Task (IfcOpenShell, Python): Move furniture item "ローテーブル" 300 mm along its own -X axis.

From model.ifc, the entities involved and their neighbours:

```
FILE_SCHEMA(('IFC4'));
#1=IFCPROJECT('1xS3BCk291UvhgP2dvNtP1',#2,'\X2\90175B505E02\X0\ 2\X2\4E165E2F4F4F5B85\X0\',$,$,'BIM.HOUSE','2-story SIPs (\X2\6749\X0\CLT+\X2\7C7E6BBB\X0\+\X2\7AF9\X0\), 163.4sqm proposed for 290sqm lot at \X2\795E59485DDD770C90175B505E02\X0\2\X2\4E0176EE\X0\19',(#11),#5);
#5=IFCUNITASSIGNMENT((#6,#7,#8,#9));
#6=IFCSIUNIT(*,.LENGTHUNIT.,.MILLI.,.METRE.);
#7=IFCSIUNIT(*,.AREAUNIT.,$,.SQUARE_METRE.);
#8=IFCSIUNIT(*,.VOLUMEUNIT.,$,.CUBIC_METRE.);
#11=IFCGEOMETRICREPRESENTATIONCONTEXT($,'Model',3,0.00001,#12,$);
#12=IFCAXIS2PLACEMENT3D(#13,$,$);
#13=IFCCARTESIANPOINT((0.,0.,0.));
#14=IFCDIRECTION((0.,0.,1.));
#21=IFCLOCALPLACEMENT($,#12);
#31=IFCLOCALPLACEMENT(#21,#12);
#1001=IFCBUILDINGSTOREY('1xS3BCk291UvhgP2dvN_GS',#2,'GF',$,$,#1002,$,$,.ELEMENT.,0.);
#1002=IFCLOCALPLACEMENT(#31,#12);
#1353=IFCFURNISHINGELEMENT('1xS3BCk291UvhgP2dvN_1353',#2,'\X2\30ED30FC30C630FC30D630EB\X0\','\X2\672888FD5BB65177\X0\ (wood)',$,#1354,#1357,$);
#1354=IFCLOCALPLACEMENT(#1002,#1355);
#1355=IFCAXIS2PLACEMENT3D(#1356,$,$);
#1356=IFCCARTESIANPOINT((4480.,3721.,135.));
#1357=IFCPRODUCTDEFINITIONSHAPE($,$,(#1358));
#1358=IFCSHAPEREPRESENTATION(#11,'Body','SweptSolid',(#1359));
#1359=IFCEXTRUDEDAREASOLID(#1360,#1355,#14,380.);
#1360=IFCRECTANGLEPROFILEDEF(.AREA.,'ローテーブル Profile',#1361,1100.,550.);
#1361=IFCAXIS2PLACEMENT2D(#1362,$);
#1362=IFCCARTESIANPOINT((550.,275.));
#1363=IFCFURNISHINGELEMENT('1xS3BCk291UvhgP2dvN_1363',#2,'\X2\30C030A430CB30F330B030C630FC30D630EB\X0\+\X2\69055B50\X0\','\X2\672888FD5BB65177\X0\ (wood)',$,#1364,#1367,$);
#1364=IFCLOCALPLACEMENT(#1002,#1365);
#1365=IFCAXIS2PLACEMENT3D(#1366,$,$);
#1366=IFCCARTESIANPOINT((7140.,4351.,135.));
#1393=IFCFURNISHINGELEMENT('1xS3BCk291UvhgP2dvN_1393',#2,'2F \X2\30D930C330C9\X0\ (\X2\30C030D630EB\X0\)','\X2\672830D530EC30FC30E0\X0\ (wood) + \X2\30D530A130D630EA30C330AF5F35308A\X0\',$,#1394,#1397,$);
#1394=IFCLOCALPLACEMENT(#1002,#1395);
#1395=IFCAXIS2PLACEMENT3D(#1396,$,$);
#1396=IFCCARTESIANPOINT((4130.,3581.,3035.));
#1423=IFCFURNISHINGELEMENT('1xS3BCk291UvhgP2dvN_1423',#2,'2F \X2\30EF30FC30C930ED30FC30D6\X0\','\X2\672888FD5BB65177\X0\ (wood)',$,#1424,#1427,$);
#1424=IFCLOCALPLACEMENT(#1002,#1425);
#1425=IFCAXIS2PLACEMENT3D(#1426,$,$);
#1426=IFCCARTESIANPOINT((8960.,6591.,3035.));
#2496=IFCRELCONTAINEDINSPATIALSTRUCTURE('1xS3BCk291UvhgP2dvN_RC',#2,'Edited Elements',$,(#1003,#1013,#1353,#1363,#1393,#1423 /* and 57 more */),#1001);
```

```python
import ifcopenshell
import ifcopenshell.api.geometry
import ifcopenshell.util.placement
import ifcopenshell.util.unit

model = ifcopenshell.open("model.ifc")
unit_scale = ifcopenshell.util.unit.calculate_unit_scale(model)

item = model.by_guid("1xS3BCk291UvhgP2dvN_1353")
matrix = ifcopenshell.util.placement.get_local_placement(item.ObjectPlacement)
matrix[:3, 3] -= matrix[:3, 0] * 0.3 / unit_scale
ifcopenshell.api.geometry.edit_object_placement(model, product=item, matrix=matrix, is_si=False)

print(ifcopenshell.util.placement.get_local_placement(item.ObjectPlacement).round(3) + 0.0)

model.write("model_rev.ifc")
```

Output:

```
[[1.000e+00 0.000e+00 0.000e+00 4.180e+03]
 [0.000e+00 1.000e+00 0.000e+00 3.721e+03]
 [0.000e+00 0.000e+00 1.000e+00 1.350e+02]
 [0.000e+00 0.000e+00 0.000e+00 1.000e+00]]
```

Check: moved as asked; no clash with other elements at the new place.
